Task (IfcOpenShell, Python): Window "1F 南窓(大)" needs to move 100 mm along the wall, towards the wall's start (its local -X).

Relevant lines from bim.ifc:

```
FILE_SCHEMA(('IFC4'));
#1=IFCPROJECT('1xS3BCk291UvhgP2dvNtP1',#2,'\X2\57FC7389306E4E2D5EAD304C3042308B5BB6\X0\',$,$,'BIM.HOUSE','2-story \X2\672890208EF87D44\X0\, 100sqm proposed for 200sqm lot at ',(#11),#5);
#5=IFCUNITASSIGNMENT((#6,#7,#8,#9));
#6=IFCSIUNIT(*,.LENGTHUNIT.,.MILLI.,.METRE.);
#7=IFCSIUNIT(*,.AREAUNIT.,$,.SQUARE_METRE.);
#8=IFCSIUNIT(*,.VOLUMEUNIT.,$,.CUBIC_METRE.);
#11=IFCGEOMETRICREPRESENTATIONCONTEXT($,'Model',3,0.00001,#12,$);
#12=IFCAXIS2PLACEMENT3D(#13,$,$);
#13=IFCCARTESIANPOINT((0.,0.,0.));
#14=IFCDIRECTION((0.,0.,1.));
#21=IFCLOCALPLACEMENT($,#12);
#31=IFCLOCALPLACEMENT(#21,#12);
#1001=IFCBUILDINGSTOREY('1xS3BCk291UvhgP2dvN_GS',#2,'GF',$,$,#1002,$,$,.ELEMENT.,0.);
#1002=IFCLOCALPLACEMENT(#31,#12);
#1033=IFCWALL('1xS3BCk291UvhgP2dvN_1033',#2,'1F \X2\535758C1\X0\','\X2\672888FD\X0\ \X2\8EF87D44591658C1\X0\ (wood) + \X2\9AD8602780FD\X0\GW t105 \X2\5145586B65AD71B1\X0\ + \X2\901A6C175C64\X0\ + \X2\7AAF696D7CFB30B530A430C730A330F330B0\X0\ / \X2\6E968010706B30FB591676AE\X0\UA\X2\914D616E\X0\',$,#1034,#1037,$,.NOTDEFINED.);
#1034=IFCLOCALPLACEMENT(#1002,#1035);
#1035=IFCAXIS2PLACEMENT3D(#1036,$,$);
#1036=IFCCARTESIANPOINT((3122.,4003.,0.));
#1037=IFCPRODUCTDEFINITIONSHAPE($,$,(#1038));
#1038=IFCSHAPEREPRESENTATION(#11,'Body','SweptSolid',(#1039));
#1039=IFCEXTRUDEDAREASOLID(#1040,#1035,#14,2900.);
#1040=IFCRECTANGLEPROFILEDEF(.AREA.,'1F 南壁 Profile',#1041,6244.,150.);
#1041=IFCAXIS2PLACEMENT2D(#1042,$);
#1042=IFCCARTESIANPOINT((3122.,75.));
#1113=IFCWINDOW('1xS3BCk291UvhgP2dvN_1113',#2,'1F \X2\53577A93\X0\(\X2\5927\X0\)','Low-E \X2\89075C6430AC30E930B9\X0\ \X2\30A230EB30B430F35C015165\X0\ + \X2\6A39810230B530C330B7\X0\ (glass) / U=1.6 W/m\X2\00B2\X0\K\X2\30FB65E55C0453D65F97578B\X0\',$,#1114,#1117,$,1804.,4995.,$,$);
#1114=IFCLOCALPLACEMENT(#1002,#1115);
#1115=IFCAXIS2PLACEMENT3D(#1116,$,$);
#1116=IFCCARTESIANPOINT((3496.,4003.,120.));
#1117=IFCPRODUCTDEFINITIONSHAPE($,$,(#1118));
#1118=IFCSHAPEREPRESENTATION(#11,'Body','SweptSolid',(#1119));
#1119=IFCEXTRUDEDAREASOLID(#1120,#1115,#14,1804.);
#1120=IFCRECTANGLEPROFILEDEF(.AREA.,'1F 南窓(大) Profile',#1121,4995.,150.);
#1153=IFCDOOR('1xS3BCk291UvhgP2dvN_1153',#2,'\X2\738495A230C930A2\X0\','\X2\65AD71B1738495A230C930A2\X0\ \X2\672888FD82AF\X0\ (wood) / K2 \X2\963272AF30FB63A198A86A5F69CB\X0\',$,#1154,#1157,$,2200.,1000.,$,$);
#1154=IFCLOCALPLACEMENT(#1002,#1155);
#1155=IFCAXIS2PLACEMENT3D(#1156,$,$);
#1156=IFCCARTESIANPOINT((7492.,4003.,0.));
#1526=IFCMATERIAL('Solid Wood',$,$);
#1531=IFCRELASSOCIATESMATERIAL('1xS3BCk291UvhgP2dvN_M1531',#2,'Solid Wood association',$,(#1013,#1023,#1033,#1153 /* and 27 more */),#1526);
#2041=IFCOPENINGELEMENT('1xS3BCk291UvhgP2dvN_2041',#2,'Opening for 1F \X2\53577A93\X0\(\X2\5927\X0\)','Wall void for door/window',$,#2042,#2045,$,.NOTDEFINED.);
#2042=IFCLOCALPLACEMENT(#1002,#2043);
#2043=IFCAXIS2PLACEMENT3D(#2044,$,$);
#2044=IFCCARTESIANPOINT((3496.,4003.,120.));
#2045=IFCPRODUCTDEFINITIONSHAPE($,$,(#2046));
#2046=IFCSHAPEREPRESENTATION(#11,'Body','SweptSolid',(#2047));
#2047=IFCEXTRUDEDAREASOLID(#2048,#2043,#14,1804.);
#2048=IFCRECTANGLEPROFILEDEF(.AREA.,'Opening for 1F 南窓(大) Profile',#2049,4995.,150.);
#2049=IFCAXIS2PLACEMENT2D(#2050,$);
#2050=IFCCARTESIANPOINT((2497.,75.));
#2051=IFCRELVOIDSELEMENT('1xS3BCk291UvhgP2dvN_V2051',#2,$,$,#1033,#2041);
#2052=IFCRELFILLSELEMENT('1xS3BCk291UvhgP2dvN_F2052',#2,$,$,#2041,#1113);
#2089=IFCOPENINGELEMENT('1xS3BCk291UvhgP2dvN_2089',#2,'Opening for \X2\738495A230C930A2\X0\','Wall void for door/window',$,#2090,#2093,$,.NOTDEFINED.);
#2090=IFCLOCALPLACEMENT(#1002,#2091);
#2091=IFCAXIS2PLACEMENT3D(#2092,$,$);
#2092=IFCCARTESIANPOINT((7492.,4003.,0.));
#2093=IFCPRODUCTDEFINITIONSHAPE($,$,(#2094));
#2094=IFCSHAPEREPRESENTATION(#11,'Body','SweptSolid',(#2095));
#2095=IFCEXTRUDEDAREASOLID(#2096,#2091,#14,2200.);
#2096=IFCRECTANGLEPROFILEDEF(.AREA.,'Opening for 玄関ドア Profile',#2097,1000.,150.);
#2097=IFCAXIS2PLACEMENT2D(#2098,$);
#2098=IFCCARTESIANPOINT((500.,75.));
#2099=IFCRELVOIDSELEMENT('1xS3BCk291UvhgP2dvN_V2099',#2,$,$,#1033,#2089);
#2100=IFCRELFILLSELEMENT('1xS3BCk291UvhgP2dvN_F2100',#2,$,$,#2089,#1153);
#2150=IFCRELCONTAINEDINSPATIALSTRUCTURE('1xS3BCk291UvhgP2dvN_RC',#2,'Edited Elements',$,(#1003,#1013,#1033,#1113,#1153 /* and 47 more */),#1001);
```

```python
import ifcopenshell
import ifcopenshell.api.geometry
import ifcopenshell.util.placement
import ifcopenshell.util.unit

model = ifcopenshell.open("bim.ifc")
unit_scale = ifcopenshell.util.unit.calculate_unit_scale(model)

window = model.by_guid("1xS3BCk291UvhgP2dvN_1113")
opening = window.FillsVoids[0].RelatingOpeningElement
wall = opening.VoidsElements[0].RelatingBuildingElement

wall_matrix = ifcopenshell.util.placement.get_local_placement(wall.ObjectPlacement)
shift = wall_matrix[:3, 0] * -0.1 / unit_scale
before = ifcopenshell.util.placement.get_local_placement(window.ObjectPlacement)[:3, 3].copy()

# The window is not placed relative to its opening, so move both.
for product in (opening, window):
    matrix = ifcopenshell.util.placement.get_local_placement(product.ObjectPlacement)
    matrix[:3, 3] += shift
    ifcopenshell.api.geometry.edit_object_placement(model, product=product, matrix=matrix, is_si=False)

after = ifcopenshell.util.placement.get_local_placement(window.ObjectPlacement)[:3, 3]
print("window moved by", (after - before).round(3) + 0.0)

model.write("bim-out.ifc")
```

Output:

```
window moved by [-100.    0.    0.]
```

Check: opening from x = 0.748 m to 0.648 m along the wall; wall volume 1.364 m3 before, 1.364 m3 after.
